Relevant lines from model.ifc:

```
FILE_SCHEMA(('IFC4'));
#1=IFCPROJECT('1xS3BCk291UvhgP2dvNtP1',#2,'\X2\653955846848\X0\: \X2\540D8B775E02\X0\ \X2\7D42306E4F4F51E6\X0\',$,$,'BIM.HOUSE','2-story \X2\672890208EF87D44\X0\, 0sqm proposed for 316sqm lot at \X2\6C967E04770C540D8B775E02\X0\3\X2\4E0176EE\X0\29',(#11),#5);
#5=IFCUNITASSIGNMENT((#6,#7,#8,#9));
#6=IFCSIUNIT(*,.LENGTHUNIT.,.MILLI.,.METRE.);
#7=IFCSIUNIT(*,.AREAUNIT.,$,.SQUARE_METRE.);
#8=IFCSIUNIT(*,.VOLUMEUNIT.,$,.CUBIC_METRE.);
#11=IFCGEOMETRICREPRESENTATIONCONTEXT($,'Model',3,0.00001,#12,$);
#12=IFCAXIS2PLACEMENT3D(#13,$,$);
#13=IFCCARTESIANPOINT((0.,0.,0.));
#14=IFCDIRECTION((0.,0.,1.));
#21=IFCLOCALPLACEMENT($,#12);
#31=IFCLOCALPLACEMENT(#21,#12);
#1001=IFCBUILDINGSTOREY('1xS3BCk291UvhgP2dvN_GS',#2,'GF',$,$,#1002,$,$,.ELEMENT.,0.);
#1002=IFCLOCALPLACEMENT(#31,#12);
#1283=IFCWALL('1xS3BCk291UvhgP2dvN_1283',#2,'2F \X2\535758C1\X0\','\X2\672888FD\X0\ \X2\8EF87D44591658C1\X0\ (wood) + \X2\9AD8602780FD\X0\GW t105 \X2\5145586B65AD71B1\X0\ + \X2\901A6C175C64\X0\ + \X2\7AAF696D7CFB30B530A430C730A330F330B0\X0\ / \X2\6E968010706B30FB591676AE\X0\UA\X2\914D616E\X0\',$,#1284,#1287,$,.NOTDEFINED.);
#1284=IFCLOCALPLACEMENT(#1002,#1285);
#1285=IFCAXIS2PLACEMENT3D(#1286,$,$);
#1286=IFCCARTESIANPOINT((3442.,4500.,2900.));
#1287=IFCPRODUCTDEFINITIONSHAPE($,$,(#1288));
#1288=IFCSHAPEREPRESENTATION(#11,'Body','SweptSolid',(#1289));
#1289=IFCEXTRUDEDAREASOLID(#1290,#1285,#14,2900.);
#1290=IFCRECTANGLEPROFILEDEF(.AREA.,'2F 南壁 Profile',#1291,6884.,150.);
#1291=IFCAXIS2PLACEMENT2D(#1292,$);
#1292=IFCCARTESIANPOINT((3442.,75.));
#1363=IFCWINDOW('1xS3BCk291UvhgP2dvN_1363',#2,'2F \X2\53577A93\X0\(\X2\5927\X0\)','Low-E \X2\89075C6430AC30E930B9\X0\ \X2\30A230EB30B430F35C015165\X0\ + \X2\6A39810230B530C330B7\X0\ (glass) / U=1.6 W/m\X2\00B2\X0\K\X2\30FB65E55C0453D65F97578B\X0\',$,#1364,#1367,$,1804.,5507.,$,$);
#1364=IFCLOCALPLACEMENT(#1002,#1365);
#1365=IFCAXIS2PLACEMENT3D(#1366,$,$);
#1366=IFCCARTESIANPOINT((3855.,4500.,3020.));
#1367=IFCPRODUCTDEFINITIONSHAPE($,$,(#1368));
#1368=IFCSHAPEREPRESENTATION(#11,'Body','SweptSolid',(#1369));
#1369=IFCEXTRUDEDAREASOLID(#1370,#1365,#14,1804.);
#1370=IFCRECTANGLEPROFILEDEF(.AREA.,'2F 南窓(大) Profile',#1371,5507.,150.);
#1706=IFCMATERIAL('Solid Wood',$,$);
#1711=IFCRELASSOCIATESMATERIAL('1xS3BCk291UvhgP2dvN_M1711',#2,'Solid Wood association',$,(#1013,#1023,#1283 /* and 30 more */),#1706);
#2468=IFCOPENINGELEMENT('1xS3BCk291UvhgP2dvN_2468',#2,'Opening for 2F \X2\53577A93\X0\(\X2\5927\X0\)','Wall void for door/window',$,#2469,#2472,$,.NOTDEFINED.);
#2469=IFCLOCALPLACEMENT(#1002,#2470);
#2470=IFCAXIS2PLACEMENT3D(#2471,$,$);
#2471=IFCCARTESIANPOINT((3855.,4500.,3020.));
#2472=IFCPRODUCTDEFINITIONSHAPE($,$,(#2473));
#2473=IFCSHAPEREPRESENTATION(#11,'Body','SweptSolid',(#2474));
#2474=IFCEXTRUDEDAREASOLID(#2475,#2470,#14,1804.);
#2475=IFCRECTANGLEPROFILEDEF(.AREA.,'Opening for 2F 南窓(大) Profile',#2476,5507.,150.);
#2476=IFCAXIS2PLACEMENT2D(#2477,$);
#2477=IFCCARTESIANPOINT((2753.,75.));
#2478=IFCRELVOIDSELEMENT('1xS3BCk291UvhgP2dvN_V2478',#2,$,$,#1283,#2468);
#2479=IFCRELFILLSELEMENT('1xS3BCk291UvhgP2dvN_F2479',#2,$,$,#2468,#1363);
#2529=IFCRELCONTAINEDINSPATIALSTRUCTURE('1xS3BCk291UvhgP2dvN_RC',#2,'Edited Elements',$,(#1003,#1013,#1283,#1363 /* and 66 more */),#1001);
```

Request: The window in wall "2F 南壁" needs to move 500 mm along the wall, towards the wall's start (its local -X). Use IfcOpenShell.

```python
import ifcopenshell
import ifcopenshell.api.geometry
import ifcopenshell.util.placement
import ifcopenshell.util.unit

model = ifcopenshell.open("model.ifc")
unit_scale = ifcopenshell.util.unit.calculate_unit_scale(model)

window = model.by_id(1363)
opening = window.FillsVoids[0].RelatingOpeningElement
wall = opening.VoidsElements[0].RelatingBuildingElement

wall_matrix = ifcopenshell.util.placement.get_local_placement(wall.ObjectPlacement)
shift = wall_matrix[:3, 0] * -0.5 / unit_scale
before = ifcopenshell.util.placement.get_local_placement(window.ObjectPlacement)[:3, 3].copy()

# The window is not placed relative to its opening, so move both.
for product in (opening, window):
    matrix = ifcopenshell.util.placement.get_local_placement(product.ObjectPlacement)
    matrix[:3, 3] += shift
    ifcopenshell.api.geometry.edit_object_placement(model, product=product, matrix=matrix, is_si=False)

after = ifcopenshell.util.placement.get_local_placement(window.ObjectPlacement)[:3, 3]
print("window moved by", (after - before).round(3) + 0.0)

model.write("model_v2.ifc")
```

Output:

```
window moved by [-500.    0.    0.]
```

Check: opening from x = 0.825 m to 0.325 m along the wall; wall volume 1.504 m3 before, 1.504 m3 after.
